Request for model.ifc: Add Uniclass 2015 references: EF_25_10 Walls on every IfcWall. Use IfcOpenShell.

First a look at what the model holds.

```python
import ifcopenshell

model = ifcopenshell.open("model.ifc")
print(model.schema)
print("classifications:", [c.Name for c in model.by_type("IfcClassification")])
for ifc_class in ("IfcDoor", "IfcRoof", "IfcStair", "IfcWall", "IfcWindow"):
    print(ifc_class, len(model.by_type(ifc_class)))
```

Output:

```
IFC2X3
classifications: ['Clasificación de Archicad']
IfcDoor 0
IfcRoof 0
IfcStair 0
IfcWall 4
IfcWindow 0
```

```python
import ifcopenshell
import ifcopenshell.api.classification

model = ifcopenshell.open("model.ifc")

# IFC2X3 requires Source and Edition and has no link from the project to the system.
system = model.create_entity("IfcClassification", Source="NBS", Edition="2015", Name="Uniclass 2015")

codes = {
    "IfcWall": ("EF_25_10", "Walls"),
}
for ifc_class, (code, name) in codes.items():
    products = model.by_type(ifc_class)
    ifcopenshell.api.classification.add_reference(
        model, products=products, classification=system, identification=code, name=name
    )
    print(code, len(products))

model.write("model_v2.ifc")
```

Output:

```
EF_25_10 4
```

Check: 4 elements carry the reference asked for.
